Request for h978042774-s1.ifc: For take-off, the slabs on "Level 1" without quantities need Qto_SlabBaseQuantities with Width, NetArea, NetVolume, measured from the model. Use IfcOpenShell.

First a look at what the model holds.

```python
import ifcopenshell
import ifcopenshell.util.element
import ifcopenshell.util.unit

model = ifcopenshell.open("h978042774-s1.ifc")
print(model.schema)
for unit_type in ("LENGTHUNIT", "AREAUNIT", "VOLUMEUNIT"):
    print(unit_type, ifcopenshell.util.unit.calculate_unit_scale(model, unit_type))
storey = next(s for s in model.by_type("IfcBuildingStorey") if s.Name == "Level 1")
slabs = [e for e in ifcopenshell.util.element.get_decomposition(storey) if e.is_a("IfcSlab")]
for e in sorted(slabs, key=lambda e: e.id()):
    print(e.id(), e.is_a(), e.Name, list(ifcopenshell.util.element.get_psets(e, qtos_only=True)), sep=" | ")
```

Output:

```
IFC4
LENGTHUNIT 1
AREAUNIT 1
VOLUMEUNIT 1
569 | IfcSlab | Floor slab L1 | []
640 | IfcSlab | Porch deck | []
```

```python
import ifcopenshell
import ifcopenshell.api.pset
import ifcopenshell.geom
import ifcopenshell.util.element
import ifcopenshell.util.shape
import ifcopenshell.util.unit

model = ifcopenshell.open("h978042774-s1.ifc")
unit_scale = ifcopenshell.util.unit.calculate_unit_scale(model)
area_scale = ifcopenshell.util.unit.calculate_unit_scale(model, "AREAUNIT")
volume_scale = ifcopenshell.util.unit.calculate_unit_scale(model, "VOLUMEUNIT")
settings = ifcopenshell.geom.settings()

storey = next(s for s in model.by_type("IfcBuildingStorey") if s.Name == "Level 1")
slabs = [e for e in ifcopenshell.util.element.get_decomposition(storey) if e.is_a("IfcSlab")]

for e in sorted(slabs, key=lambda e: e.id()):
    if ifcopenshell.util.element.get_psets(e, qtos_only=True, should_inherit=False):
        continue
    # Geometry comes back in metres, in the element's own axes.
    shape = ifcopenshell.geom.create_shape(settings, e)
    values = {
        "Width": ifcopenshell.util.shape.get_z(shape.geometry) / unit_scale,
        "NetArea": ifcopenshell.util.shape.get_footprint_area(shape.geometry) / area_scale,
        "NetVolume": ifcopenshell.util.shape.get_volume(shape.geometry) / volume_scale,
    }
    qto = ifcopenshell.api.pset.add_qto(model, product=e, name="Qto_SlabBaseQuantities")
    ifcopenshell.api.pset.edit_qto(model, qto=qto, properties=values)
    print(e.id(), {k: round(v, 3) for k, v in values.items()})

model.write("h978042774-s1_rev.ifc")
```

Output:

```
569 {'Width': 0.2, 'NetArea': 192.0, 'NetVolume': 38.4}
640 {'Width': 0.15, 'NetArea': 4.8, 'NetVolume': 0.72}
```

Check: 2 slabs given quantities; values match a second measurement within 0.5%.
